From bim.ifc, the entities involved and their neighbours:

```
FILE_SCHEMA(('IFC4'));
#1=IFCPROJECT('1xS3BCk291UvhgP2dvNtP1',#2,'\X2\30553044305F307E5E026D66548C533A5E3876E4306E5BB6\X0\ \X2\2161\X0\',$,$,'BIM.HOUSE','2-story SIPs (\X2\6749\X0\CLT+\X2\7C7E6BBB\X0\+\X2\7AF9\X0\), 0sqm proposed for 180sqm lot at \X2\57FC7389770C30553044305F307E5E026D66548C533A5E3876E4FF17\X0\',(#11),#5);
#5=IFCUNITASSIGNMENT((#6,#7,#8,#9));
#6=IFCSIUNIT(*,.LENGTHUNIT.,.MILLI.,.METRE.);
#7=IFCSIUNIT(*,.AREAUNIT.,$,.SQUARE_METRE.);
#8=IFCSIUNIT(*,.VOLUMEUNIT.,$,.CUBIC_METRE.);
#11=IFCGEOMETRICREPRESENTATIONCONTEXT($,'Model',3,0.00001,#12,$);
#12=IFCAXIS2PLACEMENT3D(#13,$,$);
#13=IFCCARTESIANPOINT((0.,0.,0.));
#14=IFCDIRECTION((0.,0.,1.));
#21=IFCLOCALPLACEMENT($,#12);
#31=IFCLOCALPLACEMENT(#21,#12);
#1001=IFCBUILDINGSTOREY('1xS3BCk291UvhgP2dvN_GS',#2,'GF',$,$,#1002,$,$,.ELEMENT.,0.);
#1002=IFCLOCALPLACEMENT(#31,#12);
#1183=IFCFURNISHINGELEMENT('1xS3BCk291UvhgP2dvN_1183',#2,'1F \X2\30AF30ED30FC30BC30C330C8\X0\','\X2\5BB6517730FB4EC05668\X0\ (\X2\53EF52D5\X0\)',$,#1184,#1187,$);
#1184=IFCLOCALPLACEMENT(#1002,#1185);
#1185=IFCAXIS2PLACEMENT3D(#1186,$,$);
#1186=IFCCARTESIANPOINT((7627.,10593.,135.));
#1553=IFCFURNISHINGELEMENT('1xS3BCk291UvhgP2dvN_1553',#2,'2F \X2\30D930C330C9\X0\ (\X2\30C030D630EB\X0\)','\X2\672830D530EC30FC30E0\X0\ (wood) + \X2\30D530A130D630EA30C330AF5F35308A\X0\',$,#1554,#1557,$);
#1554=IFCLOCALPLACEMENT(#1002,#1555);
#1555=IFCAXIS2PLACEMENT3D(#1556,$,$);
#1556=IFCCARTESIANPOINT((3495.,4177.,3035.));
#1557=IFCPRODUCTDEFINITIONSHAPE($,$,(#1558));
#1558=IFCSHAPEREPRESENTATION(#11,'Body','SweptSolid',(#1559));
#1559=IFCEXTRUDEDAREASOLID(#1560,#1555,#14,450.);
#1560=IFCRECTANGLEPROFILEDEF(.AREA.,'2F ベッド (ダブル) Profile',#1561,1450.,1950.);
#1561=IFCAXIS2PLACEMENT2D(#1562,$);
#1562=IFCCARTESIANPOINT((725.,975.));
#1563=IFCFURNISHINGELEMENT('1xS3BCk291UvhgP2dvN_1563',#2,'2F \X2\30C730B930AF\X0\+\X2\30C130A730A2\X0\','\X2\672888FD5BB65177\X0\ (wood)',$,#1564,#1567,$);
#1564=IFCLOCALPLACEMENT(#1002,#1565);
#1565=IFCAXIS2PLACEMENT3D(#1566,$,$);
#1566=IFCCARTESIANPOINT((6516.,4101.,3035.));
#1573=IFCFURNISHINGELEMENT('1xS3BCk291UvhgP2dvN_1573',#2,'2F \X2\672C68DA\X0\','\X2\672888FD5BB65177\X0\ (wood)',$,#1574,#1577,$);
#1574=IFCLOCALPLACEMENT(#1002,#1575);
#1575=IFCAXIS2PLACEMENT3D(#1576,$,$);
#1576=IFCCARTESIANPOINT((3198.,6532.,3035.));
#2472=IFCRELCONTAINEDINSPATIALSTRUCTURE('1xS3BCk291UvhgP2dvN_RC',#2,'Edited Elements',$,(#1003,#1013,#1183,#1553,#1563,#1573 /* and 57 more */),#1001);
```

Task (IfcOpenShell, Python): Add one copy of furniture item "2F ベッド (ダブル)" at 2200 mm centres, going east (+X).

```python
import numpy as np
import ifcopenshell
import ifcopenshell.api.geometry
import ifcopenshell.api.root
import ifcopenshell.util.element
import ifcopenshell.util.placement
import ifcopenshell.util.unit

model = ifcopenshell.open("bim.ifc")
unit_scale = ifcopenshell.util.unit.calculate_unit_scale(model)


def reuse_history(source, copy):
    """copy_class also copies each property set's owner history, people and application; keep the originals."""
    for rel in copy.IsDefinedBy:
        if rel.is_a("IfcRelDefinesByProperties") and (history := rel.RelatingPropertyDefinition.OwnerHistory):
            rel.RelatingPropertyDefinition.OwnerHistory = source.OwnerHistory
            ifcopenshell.util.element.remove_deep2(model, history)


source = model.by_guid("1xS3BCk291UvhgP2dvN_1553")
base = ifcopenshell.util.placement.get_local_placement(source.ObjectPlacement)
step = np.array([1.0, 0.0, 0.0]) * 2.2 / unit_scale

for i in range(1, 2):
    copy = ifcopenshell.api.root.copy_class(model, product=source)
    copy.Representation = ifcopenshell.util.element.copy_deep(
        model, source.Representation, exclude=["IfcGeometricRepresentationContext", "IfcRepresentationMap"]
    )
    reuse_history(source, copy)
    matrix = base.copy()
    matrix[:3, 3] += i * step
    print("added at", matrix[:3, 3].round(3) + 0.0)
    ifcopenshell.api.geometry.edit_object_placement(model, product=copy, matrix=matrix, is_si=False)

model.write("bim-out.ifc")
```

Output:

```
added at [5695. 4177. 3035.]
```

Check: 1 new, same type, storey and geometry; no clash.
